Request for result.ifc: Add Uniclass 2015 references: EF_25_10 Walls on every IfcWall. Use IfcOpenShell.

First a look at what the model holds.

```python
import ifcopenshell

model = ifcopenshell.open("result.ifc")
print(model.schema)
print("classifications:", [c.Name for c in model.by_type("IfcClassification")])
for ifc_class in ("IfcDoor", "IfcRoof", "IfcStair", "IfcWall", "IfcWindow"):
    print(ifc_class, len(model.by_type(ifc_class)))
```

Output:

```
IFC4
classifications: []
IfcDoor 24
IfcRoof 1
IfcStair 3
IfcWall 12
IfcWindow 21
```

```python
import ifcopenshell
import ifcopenshell.api.classification

model = ifcopenshell.open("result.ifc")

system = ifcopenshell.api.classification.add_classification(model, classification="Uniclass 2015")

codes = {
    "IfcWall": ("EF_25_10", "Walls"),
}
for ifc_class, (code, name) in codes.items():
    products = model.by_type(ifc_class)
    ifcopenshell.api.classification.add_reference(
        model, products=products, classification=system, identification=code, name=name
    )
    print(code, len(products))

model.write("result_rev.ifc")
```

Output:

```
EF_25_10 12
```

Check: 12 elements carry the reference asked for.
